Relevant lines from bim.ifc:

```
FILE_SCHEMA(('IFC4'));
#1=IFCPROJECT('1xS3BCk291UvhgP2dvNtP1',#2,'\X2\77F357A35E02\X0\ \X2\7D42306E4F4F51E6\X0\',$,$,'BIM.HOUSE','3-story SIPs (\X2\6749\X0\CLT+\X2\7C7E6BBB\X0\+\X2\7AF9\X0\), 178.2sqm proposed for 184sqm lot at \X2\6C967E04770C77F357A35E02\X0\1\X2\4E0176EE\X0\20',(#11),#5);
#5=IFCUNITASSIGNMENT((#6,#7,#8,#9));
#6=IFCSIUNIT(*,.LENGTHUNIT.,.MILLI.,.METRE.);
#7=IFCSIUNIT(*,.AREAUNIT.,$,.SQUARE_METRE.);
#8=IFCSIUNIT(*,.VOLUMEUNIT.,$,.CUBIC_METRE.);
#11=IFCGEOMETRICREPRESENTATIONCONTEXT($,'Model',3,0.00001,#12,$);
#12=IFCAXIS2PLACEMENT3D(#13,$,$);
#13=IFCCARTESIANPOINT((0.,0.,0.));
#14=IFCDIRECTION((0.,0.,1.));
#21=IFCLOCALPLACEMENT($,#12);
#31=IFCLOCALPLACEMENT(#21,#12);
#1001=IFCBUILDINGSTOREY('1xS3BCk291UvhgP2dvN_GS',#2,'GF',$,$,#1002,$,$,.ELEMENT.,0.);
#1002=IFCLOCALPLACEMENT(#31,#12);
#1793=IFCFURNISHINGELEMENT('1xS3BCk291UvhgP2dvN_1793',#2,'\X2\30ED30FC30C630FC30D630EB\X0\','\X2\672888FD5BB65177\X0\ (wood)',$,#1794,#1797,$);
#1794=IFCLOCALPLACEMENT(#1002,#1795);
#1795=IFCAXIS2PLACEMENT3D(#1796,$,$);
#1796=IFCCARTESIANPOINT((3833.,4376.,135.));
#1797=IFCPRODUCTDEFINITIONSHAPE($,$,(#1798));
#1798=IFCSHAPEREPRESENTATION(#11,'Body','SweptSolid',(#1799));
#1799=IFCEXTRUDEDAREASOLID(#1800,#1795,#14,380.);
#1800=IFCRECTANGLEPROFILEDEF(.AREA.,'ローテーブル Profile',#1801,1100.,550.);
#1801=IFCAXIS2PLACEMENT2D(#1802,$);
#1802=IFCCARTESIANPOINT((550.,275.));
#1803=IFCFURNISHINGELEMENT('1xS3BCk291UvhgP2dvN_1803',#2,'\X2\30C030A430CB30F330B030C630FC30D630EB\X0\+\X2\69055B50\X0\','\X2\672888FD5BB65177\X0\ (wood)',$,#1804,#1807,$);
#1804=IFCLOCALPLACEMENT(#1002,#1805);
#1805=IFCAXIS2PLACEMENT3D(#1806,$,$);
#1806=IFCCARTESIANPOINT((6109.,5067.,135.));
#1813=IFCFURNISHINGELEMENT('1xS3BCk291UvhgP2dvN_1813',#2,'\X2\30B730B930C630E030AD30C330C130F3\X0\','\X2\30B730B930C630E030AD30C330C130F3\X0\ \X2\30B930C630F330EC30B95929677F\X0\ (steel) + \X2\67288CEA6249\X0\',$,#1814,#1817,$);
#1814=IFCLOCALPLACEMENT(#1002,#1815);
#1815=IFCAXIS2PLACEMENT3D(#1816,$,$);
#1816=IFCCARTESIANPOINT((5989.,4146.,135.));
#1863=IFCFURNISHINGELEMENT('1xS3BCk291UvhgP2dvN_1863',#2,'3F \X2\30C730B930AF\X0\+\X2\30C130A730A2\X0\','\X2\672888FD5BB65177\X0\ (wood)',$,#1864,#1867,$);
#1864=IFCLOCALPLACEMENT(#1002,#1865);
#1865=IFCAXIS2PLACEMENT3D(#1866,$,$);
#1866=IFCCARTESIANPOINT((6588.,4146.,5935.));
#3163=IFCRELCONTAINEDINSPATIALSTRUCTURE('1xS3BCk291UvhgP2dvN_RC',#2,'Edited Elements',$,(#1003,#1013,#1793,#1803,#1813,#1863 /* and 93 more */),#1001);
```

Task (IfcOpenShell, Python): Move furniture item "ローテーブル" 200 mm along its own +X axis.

```python
import ifcopenshell
import ifcopenshell.api.geometry
import ifcopenshell.util.placement

model = ifcopenshell.open("bim.ifc")

item = model.by_id(1793)
matrix = ifcopenshell.util.placement.get_local_placement(item.ObjectPlacement)
matrix[:3, 3] += matrix[:3, 0] * 200.0
ifcopenshell.api.geometry.edit_object_placement(model, product=item, matrix=matrix, is_si=False)

print(ifcopenshell.util.placement.get_local_placement(item.ObjectPlacement).round(3) + 0.0)

model.write("bim_rev.ifc")
```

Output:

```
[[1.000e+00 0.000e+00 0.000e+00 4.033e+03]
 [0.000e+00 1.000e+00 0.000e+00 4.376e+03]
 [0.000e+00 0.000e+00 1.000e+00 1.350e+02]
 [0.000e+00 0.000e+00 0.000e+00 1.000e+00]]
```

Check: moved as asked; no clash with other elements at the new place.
